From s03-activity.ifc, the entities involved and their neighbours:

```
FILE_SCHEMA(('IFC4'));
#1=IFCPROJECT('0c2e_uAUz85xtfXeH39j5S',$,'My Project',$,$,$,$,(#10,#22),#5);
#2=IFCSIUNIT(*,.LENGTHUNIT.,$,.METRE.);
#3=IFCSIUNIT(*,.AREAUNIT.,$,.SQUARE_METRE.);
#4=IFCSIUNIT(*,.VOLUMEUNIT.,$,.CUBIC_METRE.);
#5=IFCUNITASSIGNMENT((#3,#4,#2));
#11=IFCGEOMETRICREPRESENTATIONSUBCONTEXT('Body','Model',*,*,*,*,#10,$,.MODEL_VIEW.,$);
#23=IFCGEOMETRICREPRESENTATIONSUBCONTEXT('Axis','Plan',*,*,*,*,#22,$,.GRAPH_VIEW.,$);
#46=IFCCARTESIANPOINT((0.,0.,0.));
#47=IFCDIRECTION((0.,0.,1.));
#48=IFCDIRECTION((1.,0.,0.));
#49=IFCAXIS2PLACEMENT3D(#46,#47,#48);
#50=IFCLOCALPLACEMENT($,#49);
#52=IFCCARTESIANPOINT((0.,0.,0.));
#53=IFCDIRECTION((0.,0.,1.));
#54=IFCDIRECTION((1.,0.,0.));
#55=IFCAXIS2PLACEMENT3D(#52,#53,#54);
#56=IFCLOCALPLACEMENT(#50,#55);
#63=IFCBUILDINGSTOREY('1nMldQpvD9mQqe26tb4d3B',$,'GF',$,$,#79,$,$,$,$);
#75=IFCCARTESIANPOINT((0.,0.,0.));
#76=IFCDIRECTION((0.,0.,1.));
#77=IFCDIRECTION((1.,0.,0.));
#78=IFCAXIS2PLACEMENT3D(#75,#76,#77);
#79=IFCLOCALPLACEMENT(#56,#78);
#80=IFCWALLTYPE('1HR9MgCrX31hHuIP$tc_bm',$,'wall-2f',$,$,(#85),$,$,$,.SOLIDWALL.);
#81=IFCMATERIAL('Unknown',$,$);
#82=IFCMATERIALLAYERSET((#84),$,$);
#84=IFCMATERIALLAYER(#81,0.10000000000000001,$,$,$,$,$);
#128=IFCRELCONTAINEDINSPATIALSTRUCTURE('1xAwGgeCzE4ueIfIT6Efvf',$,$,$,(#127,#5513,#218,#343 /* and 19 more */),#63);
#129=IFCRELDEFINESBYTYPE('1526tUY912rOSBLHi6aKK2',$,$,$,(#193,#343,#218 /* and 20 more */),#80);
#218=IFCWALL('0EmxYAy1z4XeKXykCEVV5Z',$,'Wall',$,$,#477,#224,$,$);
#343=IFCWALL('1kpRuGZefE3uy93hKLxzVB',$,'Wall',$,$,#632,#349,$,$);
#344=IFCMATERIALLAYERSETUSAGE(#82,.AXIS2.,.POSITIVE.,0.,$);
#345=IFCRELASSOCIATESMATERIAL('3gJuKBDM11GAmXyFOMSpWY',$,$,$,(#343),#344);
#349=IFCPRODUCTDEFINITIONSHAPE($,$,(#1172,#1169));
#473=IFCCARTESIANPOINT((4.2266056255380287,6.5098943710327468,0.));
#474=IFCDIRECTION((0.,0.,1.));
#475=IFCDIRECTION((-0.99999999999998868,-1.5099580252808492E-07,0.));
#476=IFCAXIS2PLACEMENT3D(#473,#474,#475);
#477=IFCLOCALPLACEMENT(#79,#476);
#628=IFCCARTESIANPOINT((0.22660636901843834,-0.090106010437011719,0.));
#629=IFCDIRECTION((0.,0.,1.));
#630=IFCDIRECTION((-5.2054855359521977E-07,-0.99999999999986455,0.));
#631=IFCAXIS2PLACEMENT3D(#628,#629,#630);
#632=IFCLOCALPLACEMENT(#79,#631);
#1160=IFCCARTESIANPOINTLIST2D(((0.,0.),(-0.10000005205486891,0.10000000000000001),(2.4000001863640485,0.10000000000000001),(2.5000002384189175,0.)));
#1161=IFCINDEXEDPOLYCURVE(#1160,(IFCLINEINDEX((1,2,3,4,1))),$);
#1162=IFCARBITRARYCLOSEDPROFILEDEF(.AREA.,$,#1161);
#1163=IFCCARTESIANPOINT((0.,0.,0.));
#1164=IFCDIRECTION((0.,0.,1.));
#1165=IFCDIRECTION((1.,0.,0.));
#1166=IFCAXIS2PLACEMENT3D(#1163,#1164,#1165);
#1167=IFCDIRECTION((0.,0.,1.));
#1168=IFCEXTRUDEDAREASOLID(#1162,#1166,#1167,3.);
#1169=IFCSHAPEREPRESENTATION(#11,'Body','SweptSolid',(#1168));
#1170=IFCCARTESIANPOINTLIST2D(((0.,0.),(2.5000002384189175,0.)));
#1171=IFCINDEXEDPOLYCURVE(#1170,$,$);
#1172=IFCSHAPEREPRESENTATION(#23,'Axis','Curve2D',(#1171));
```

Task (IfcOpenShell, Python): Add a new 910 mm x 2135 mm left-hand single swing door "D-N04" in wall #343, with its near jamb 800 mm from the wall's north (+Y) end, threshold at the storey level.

```python
import numpy as np
import ifcopenshell
import ifcopenshell.api.feature
import ifcopenshell.api.geometry
import ifcopenshell.api.root
import ifcopenshell.api.spatial
import ifcopenshell.geom
import ifcopenshell.util.element
import ifcopenshell.util.placement
import ifcopenshell.util.representation
import ifcopenshell.util.shape
import ifcopenshell.util.unit

model = ifcopenshell.open("s03-activity.ifc")
unit_scale = ifcopenshell.util.unit.calculate_unit_scale(model)
settings = ifcopenshell.geom.settings()


def volume(element):
    """Net volume in cubic metres, openings subtracted."""
    shape = ifcopenshell.geom.create_shape(settings, element)
    return ifcopenshell.util.shape.get_volume(shape.geometry)


wall = model.by_guid("1kpRuGZefE3uy93hKLxzVB")
storey = ifcopenshell.util.element.get_container(wall, ifc_class="IfcBuildingStorey")
context = ifcopenshell.util.representation.get_context(model, "Model", "Body", "MODEL_VIEW")
before = volume(wall)

width, height, from_end, sill = 0.91, 2.135, 0.8, 0.0  # metres

# The wall runs along its own X axis, and the end named is its -X end.
wall_shape = ifcopenshell.geom.create_shape(settings, wall)
x, y, z = ifcopenshell.util.shape.get_vertices(wall_shape.geometry).T
start = x.min() + from_end
face, thickness = float(y.min()), float(y.max() - y.min())
wall_matrix = ifcopenshell.util.placement.get_local_placement(wall.ObjectPlacement)
level = ifcopenshell.util.placement.get_local_placement(storey.ObjectPlacement)[2, 3]


def in_wall(x, y):
    """Placement at x, y metres in the wall's axes, at sill height."""
    matrix = wall_matrix.copy()
    matrix[:, 3] = wall_matrix @ np.array([x / unit_scale, y / unit_scale, 0.0, 1.0])
    matrix[2, 3] = level + sill / unit_scale
    return matrix


# Opening: a box that overshoots both wall faces by 50 mm.
opening = ifcopenshell.api.root.create_entity(model, ifc_class="IfcOpeningElement", predefined_type="OPENING")
box = ifcopenshell.api.geometry.add_wall_representation(
    model, context=context, length=width, height=height, thickness=thickness + 0.1
)
ifcopenshell.api.geometry.assign_representation(model, product=opening, representation=box)
ifcopenshell.api.geometry.edit_object_placement(model, product=opening, matrix=in_wall(start, face - 0.05), is_si=False)
ifcopenshell.api.feature.add_feature(model, feature=opening, element=wall)

door = ifcopenshell.api.root.create_entity(model, ifc_class="IfcDoor", name="D-N04", predefined_type="DOOR")
door.OverallWidth, door.OverallHeight = width / unit_scale, height / unit_scale
door.OperationType = "SINGLE_SWING_LEFT"
body = ifcopenshell.api.geometry.add_door_representation(
    model,
    context=context,
    overall_width=door.OverallWidth,
    overall_height=door.OverallHeight,
    operation_type="SINGLE_SWING_LEFT",
    lining_properties={"LiningDepth": thickness / unit_scale, "ThresholdDepth": thickness / unit_scale},
)
ifcopenshell.api.geometry.assign_representation(model, product=door, representation=body)
ifcopenshell.api.spatial.assign_container(model, products=[door], relating_structure=storey)
ifcopenshell.api.feature.add_filling(model, opening=opening, element=door)

# The lining spans the wall, so the door starts at the wall face.
ifcopenshell.api.geometry.edit_object_placement(model, product=door, matrix=in_wall(start, face), is_si=False)

after = volume(wall)

print(f"wall volume {before:.3f} -> {after:.3f} m3")

model.write("s03-activity-out.ifc")
```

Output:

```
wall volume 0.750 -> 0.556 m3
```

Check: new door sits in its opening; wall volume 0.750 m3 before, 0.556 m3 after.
